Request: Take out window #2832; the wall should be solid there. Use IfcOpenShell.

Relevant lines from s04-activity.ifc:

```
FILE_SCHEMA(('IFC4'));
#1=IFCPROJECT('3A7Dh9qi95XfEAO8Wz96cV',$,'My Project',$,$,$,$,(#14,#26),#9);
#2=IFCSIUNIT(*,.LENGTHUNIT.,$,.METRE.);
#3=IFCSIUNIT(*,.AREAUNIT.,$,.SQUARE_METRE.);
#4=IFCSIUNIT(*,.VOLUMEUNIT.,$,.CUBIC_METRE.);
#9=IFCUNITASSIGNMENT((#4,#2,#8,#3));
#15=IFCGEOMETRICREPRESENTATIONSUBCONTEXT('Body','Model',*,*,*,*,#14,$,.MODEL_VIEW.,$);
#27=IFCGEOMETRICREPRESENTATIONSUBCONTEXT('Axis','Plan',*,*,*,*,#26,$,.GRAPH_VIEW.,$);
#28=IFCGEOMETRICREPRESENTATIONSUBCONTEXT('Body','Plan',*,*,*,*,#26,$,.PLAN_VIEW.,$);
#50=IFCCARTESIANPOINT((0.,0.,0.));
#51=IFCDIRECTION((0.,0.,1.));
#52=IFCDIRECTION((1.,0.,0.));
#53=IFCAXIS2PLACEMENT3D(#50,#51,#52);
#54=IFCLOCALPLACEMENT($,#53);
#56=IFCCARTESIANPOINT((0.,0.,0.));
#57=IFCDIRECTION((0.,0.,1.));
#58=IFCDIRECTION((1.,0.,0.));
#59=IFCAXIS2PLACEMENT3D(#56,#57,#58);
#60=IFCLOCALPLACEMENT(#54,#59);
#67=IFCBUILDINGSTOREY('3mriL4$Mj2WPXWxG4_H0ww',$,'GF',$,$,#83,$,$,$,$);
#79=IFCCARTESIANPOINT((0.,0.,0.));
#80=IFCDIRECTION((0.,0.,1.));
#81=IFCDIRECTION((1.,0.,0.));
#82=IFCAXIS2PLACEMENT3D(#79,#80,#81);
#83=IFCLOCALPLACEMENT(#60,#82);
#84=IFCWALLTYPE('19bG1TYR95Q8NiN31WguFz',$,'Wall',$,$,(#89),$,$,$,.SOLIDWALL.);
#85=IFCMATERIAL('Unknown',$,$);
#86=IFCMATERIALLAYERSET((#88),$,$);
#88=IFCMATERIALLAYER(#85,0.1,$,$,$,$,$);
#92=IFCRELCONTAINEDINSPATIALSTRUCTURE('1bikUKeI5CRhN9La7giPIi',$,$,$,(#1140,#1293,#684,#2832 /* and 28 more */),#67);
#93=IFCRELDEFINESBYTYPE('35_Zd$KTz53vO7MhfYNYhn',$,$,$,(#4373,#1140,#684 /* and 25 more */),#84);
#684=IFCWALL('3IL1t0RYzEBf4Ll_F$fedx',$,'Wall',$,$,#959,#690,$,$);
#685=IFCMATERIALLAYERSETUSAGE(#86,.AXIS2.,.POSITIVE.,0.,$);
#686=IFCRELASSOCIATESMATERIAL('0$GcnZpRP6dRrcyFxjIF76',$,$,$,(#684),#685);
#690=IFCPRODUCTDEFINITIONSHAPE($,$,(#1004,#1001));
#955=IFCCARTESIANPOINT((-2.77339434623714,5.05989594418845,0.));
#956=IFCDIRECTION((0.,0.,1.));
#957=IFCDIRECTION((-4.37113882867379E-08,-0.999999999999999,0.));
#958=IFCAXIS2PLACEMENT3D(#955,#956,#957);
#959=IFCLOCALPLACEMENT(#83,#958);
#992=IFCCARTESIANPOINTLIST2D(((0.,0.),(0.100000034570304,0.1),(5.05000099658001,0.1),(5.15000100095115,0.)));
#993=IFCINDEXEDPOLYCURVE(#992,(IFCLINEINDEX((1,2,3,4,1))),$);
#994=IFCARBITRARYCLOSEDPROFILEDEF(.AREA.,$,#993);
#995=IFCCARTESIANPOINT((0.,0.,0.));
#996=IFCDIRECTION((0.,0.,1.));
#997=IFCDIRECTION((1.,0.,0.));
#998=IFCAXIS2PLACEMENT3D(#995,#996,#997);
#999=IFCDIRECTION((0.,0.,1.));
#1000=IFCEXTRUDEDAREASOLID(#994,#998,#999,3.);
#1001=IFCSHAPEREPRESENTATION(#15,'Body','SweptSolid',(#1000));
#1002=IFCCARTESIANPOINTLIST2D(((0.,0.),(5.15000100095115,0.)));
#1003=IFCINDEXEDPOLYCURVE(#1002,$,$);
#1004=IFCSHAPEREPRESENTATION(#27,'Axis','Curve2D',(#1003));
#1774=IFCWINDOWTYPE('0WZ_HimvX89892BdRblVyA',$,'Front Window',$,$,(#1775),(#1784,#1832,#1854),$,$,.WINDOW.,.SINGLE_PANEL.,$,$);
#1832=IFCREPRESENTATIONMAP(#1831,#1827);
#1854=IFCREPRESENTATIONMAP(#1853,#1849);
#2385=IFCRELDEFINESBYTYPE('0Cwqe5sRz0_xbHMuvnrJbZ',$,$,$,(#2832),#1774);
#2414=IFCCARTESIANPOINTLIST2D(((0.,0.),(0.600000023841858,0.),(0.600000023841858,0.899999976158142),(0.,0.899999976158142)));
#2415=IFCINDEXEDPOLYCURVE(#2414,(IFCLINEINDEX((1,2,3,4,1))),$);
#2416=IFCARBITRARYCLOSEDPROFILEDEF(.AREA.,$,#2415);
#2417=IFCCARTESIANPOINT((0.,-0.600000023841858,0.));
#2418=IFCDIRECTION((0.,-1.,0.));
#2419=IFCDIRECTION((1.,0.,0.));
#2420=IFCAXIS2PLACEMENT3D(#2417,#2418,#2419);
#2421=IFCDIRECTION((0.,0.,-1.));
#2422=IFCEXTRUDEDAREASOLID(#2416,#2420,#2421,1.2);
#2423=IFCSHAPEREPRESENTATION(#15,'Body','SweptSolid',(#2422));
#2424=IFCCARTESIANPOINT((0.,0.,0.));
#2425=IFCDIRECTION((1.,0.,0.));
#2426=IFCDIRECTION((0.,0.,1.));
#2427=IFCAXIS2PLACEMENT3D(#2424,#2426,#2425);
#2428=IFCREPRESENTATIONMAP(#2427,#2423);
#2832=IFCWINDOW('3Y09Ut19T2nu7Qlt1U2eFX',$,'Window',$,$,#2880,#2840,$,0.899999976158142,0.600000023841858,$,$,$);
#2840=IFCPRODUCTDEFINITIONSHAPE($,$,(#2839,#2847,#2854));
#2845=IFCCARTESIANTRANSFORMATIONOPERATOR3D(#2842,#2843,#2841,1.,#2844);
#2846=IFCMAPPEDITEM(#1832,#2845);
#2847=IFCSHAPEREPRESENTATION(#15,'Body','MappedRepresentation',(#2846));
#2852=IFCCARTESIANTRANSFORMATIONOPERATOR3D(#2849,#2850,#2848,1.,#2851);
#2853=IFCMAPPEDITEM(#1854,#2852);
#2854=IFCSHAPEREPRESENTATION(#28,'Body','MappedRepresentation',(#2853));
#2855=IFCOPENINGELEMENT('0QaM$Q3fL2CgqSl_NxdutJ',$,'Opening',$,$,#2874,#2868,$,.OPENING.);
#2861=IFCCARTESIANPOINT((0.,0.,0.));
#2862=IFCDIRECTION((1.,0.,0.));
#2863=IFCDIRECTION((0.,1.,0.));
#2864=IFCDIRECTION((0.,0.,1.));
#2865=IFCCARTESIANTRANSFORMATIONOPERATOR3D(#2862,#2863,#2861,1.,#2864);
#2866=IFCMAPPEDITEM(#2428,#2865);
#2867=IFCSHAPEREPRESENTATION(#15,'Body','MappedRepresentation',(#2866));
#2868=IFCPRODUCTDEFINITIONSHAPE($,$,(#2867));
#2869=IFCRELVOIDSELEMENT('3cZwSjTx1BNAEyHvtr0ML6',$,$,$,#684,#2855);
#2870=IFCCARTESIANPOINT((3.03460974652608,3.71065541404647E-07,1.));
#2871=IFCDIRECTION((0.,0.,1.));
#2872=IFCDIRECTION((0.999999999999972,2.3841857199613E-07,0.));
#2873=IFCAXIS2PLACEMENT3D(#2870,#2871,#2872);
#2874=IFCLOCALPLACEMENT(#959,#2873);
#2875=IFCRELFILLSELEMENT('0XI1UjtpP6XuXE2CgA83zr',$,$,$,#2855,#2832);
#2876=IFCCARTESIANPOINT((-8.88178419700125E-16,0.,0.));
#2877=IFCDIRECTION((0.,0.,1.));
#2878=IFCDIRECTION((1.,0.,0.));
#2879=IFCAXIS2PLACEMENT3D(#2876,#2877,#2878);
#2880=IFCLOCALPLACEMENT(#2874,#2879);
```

```python
import ifcopenshell
import ifcopenshell.api.feature
import ifcopenshell.api.root
import ifcopenshell.geom
import ifcopenshell.util.shape

model = ifcopenshell.open("s04-activity.ifc")
settings = ifcopenshell.geom.settings()


def volume(element):
    """Net volume in cubic metres, openings subtracted."""
    shape = ifcopenshell.geom.create_shape(settings, element)
    return ifcopenshell.util.shape.get_volume(shape.geometry)


window = model.by_guid("3Y09Ut19T2nu7Qlt1U2eFX")
opening = window.FillsVoids[0].RelatingOpeningElement
wall = opening.VoidsElements[0].RelatingBuildingElement
before = volume(wall)

ifcopenshell.api.root.remove_product(model, product=window)
ifcopenshell.api.feature.remove_feature(model, feature=opening)

after = volume(wall)

print(f"wall volume {before:.3f} -> {after:.3f} m3")

model.write("s04-activity-out.ifc")
```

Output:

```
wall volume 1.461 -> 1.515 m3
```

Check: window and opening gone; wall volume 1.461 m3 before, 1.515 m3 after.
